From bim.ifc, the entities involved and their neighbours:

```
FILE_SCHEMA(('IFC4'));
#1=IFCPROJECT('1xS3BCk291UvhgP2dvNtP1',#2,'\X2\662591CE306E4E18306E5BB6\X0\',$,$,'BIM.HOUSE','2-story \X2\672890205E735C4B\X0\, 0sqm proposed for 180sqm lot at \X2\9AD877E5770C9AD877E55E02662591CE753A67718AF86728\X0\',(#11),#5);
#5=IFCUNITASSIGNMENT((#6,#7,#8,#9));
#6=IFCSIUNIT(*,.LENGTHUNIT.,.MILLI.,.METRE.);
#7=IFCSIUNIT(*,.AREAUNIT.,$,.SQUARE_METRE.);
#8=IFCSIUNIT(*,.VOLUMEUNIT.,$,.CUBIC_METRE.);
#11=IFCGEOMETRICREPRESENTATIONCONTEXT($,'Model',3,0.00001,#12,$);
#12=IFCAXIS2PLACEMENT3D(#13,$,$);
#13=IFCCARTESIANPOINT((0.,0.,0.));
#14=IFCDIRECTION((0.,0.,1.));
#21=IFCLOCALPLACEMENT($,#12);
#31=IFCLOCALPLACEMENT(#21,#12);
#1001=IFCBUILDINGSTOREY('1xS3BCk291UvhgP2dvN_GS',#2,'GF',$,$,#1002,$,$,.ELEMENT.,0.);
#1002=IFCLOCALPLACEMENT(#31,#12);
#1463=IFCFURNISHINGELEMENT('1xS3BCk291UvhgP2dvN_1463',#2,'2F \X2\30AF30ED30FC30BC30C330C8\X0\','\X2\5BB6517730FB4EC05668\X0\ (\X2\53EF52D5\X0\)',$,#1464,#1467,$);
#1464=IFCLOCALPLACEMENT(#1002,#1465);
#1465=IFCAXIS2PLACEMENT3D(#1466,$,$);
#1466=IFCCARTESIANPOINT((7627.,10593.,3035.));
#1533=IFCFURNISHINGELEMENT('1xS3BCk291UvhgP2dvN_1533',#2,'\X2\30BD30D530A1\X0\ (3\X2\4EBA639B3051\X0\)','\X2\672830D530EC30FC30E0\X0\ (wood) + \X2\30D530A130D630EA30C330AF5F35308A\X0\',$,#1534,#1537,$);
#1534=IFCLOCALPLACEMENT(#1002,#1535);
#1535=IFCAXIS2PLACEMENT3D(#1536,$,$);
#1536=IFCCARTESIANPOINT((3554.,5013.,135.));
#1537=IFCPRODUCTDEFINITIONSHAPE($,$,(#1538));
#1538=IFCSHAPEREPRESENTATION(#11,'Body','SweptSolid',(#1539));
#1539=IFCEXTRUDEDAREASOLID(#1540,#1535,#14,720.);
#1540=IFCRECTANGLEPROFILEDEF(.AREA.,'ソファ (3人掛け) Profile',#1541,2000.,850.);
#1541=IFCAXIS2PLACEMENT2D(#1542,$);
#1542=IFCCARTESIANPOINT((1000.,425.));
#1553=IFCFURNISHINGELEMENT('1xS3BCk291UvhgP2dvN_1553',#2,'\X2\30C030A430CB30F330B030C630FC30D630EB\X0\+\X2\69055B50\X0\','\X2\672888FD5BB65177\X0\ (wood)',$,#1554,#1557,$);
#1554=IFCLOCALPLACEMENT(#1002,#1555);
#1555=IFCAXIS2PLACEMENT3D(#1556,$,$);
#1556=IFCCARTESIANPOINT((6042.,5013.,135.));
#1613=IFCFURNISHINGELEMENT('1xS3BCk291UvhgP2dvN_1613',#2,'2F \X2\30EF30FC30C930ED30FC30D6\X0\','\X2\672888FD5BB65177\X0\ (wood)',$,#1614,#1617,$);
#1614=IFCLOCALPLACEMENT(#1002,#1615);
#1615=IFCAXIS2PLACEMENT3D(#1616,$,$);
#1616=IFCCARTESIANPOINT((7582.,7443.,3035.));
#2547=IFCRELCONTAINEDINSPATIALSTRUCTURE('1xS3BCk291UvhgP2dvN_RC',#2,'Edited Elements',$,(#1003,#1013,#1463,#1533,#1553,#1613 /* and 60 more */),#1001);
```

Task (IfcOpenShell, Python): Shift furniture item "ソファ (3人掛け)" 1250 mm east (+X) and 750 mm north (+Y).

```python
import ifcopenshell
import ifcopenshell.api.geometry
import ifcopenshell.util.placement

model = ifcopenshell.open("bim.ifc")

item = model.by_guid("1xS3BCk291UvhgP2dvN_1533")
matrix = ifcopenshell.util.placement.get_local_placement(item.ObjectPlacement)
matrix[0, 3] += 1250.0
matrix[1, 3] += 750.0
ifcopenshell.api.geometry.edit_object_placement(model, product=item, matrix=matrix, is_si=False)

print(ifcopenshell.util.placement.get_local_placement(item.ObjectPlacement).round(3) + 0.0)

model.write("bim_updated.ifc")
```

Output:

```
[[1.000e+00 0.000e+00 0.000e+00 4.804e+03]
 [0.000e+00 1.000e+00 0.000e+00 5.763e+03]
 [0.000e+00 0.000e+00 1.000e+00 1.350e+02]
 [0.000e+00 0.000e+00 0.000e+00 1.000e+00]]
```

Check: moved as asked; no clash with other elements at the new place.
